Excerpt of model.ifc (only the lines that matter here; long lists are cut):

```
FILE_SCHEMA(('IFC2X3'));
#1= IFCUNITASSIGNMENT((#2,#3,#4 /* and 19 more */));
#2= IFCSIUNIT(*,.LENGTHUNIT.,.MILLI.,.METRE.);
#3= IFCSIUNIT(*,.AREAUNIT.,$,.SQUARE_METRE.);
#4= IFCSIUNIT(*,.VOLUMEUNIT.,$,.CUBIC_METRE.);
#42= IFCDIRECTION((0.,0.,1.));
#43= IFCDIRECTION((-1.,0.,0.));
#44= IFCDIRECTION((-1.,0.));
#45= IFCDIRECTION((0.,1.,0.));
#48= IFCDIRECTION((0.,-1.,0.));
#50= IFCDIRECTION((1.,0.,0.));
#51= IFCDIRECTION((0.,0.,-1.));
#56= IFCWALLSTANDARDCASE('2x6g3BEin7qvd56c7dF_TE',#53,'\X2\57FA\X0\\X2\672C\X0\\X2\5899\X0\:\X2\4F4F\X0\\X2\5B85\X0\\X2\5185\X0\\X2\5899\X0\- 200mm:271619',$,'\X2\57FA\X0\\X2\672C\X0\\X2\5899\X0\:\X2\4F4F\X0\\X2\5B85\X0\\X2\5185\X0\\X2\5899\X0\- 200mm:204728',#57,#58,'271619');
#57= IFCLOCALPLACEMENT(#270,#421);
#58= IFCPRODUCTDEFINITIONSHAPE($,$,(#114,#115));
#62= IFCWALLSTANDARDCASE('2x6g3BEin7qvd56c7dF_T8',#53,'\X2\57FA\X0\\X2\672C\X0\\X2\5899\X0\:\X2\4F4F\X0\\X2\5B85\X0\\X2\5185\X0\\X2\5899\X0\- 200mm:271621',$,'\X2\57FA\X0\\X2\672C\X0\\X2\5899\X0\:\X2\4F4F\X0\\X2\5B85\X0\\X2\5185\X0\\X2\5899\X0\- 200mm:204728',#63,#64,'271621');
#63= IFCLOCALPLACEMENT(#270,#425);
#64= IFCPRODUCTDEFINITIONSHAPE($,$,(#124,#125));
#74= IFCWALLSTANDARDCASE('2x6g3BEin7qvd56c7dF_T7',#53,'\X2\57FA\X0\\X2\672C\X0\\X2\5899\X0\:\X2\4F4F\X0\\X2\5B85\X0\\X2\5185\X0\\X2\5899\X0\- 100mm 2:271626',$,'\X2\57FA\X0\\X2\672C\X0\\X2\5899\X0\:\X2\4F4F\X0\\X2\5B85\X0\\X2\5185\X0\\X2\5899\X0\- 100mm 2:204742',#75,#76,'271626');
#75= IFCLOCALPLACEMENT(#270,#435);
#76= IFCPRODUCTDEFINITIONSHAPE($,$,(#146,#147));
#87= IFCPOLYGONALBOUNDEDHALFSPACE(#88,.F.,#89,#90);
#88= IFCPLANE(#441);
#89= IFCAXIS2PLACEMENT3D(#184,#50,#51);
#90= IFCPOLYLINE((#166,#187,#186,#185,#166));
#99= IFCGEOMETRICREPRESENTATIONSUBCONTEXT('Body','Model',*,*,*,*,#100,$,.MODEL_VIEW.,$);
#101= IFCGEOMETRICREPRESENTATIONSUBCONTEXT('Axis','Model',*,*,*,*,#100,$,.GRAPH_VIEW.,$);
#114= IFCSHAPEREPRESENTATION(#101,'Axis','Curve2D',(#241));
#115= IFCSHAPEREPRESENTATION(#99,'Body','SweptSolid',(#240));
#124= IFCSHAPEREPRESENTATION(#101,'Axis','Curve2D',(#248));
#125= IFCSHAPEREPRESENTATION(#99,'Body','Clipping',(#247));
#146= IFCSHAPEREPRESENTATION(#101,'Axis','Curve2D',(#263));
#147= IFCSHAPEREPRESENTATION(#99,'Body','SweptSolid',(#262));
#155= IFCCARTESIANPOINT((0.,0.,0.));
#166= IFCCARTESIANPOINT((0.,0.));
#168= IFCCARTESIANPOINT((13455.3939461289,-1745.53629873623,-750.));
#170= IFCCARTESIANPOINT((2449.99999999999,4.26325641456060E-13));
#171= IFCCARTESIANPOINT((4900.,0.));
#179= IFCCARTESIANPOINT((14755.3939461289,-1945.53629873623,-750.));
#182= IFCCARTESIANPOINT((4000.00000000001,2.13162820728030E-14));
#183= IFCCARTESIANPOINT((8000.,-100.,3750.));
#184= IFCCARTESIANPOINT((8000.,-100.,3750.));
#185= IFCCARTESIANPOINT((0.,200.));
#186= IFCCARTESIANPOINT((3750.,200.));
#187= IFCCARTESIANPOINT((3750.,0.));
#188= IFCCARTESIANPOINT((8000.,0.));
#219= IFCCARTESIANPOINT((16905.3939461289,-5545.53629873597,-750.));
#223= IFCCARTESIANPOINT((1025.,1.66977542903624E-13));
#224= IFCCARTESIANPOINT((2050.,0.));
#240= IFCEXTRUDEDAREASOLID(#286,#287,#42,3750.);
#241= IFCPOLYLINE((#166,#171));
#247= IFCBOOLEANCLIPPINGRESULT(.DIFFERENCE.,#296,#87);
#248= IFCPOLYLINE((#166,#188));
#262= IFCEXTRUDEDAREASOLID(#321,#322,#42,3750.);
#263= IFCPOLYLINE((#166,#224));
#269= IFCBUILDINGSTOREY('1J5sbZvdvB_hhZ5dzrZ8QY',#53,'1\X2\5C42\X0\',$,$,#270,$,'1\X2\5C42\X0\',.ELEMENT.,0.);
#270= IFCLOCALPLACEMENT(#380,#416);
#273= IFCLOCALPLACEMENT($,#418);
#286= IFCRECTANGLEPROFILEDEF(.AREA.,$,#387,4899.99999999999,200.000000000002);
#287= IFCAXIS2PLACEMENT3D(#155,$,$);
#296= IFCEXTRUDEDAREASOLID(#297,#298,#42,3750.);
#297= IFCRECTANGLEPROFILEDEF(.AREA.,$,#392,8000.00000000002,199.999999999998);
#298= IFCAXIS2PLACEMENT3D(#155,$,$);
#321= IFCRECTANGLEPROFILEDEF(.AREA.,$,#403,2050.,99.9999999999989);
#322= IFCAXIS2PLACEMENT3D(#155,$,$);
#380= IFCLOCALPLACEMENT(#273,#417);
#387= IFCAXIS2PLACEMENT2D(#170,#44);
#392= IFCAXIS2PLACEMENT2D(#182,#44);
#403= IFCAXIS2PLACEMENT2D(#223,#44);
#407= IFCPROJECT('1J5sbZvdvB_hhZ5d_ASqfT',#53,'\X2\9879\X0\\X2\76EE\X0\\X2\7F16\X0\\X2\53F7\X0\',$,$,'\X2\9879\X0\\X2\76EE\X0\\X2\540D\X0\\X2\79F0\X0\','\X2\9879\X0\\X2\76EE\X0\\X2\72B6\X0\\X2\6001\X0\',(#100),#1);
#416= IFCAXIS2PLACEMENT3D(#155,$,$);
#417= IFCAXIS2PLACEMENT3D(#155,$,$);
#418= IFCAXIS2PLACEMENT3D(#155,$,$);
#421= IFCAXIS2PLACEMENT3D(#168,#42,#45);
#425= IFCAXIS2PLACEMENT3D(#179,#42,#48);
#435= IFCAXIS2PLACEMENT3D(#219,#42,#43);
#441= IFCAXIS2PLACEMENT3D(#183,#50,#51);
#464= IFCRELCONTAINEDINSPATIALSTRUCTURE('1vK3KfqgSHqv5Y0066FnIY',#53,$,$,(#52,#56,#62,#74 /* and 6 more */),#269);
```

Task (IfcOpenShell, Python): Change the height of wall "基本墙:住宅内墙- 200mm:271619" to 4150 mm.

```python
import ifcopenshell
import ifcopenshell.geom
import ifcopenshell.util.representation
import ifcopenshell.util.shape
import ifcopenshell.util.unit

model = ifcopenshell.open("model.ifc")
unit_scale = ifcopenshell.util.unit.calculate_unit_scale(model)
settings = ifcopenshell.geom.settings()


def volume(element):
    """Net volume in cubic metres, openings subtracted."""
    shape = ifcopenshell.geom.create_shape(settings, element)
    return ifcopenshell.util.shape.get_volume(shape.geometry)


wall = model.by_id(56)
before = volume(wall)

body = ifcopenshell.util.representation.get_representation(wall, "Model", "Body")
solid = body.Items[0]
old_height = solid.Depth
solid.Depth = 4.15 / unit_scale
after = volume(wall)

print(f"height {old_height:g} -> {solid.Depth:g}, volume {before:.3f} -> {after:.3f} m3")

model.write("model_rev.ifc")
```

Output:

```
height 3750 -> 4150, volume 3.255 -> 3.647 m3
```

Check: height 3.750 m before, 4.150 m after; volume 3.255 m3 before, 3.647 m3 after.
